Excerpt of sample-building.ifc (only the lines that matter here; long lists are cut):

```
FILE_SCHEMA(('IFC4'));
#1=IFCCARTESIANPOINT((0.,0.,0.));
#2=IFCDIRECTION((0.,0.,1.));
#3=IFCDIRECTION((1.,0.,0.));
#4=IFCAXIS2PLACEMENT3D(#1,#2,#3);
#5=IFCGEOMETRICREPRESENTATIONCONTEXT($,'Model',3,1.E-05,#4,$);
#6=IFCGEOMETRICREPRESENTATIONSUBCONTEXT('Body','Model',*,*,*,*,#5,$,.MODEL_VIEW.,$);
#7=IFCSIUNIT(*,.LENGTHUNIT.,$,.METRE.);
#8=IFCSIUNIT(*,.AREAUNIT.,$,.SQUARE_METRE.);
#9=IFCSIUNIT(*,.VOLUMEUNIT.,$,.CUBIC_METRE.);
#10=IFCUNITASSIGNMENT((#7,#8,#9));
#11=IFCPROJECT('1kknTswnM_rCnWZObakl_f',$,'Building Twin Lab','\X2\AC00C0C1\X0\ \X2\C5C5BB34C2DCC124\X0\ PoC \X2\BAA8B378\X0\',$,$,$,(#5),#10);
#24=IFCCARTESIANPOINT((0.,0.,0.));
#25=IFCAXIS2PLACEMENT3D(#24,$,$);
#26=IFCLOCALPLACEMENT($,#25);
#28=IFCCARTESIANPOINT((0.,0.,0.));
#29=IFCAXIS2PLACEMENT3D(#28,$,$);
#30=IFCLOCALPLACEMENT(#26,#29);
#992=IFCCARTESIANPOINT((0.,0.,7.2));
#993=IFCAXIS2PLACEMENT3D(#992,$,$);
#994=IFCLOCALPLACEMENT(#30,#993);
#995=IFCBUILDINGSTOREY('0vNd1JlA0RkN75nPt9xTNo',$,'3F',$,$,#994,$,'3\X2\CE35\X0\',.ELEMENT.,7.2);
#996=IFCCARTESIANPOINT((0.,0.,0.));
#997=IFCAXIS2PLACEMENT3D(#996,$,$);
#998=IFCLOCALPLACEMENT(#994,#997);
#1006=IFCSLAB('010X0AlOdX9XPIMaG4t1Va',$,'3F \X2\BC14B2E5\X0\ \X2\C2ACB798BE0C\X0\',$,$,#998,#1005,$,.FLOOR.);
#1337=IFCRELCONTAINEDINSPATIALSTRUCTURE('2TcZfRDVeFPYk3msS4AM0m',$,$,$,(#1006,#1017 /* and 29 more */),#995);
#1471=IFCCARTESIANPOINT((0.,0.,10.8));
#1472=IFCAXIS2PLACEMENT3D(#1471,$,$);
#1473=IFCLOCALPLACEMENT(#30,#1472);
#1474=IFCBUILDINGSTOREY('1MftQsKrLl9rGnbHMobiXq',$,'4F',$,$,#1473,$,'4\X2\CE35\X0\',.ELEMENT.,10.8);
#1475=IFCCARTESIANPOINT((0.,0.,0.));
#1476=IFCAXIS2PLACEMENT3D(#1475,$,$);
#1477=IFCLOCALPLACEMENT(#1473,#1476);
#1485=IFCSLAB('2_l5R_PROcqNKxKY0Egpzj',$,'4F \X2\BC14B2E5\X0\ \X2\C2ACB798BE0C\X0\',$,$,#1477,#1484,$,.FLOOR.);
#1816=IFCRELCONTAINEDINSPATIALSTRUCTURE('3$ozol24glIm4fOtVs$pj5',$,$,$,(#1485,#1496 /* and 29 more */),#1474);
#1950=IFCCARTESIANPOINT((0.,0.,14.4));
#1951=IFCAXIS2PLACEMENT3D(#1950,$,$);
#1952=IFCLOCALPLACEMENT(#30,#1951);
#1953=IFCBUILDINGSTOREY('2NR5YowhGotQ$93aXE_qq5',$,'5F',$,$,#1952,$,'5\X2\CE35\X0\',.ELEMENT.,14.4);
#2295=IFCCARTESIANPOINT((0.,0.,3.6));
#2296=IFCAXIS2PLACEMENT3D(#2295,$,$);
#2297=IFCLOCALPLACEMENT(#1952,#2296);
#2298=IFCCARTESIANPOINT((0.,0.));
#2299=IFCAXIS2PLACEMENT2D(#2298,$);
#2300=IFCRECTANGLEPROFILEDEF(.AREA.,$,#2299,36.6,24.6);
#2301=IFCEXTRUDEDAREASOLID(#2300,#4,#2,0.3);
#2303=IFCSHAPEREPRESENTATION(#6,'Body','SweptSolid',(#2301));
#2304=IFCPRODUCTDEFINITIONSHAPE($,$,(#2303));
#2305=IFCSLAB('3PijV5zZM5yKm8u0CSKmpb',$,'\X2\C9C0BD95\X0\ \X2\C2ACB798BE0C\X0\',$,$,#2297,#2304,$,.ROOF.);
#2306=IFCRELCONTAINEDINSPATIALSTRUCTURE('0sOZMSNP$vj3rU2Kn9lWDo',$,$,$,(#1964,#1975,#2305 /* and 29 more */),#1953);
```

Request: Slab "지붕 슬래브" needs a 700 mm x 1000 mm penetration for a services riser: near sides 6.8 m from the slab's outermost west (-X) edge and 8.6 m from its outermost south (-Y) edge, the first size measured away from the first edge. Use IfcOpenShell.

```python
import numpy as np
import ifcopenshell
import ifcopenshell.api.feature
import ifcopenshell.api.geometry
import ifcopenshell.api.root
import ifcopenshell.geom
import ifcopenshell.util.placement
import ifcopenshell.util.representation
import ifcopenshell.util.shape
import ifcopenshell.util.unit

model = ifcopenshell.open("sample-building.ifc")
unit_scale = ifcopenshell.util.unit.calculate_unit_scale(model)
settings = ifcopenshell.geom.settings()


def volume(element):
    """Net volume in cubic metres, openings subtracted."""
    shape = ifcopenshell.geom.create_shape(settings, element)
    return ifcopenshell.util.shape.get_volume(shape.geometry)


slab = model.by_guid("3PijV5zZM5yKm8u0CSKmpb")
before = volume(slab)

# Extent in the slab's own axes, in metres. The edges named are its -X and -Y sides.
slab_shape = ifcopenshell.geom.create_shape(settings, slab)
vertices = ifcopenshell.util.shape.get_vertices(slab_shape.geometry)
x_min, y_min, bottom = vertices.min(axis=0)
top = vertices[:, 2].max()

opening = ifcopenshell.api.root.create_entity(model, ifc_class="IfcOpeningElement", name="Services riser opening", predefined_type="OPENING")
context = ifcopenshell.util.representation.get_context(model, "Model", "Body", "MODEL_VIEW")
width, depth = 0.7, 1
outline = [(0.0, 0.0), (width, 0.0), (width, depth), (0.0, depth), (0.0, 0.0)]
# Overshoot both faces by 50 mm so the cut is clean.
shape = ifcopenshell.api.geometry.add_slab_representation(
    model, context=context, depth=top - bottom + 0.1, polyline=outline
)
ifcopenshell.api.geometry.assign_representation(model, product=opening, representation=shape)

matrix = ifcopenshell.util.placement.get_local_placement(slab.ObjectPlacement)
matrix[:, 3] = matrix @ np.append(np.array([x_min + 6.8, y_min + 8.6, bottom - 0.05]) / unit_scale, 1.0)
ifcopenshell.api.geometry.edit_object_placement(model, product=opening, matrix=matrix, is_si=False)
ifcopenshell.api.feature.add_feature(model, feature=opening, element=slab)

after = volume(slab)

print(f"slab volume {before:.3f} -> {after:.3f} m3")

model.write("sample-building_updated.ifc")
```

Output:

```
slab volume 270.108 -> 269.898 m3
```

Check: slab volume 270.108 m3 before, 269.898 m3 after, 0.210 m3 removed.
